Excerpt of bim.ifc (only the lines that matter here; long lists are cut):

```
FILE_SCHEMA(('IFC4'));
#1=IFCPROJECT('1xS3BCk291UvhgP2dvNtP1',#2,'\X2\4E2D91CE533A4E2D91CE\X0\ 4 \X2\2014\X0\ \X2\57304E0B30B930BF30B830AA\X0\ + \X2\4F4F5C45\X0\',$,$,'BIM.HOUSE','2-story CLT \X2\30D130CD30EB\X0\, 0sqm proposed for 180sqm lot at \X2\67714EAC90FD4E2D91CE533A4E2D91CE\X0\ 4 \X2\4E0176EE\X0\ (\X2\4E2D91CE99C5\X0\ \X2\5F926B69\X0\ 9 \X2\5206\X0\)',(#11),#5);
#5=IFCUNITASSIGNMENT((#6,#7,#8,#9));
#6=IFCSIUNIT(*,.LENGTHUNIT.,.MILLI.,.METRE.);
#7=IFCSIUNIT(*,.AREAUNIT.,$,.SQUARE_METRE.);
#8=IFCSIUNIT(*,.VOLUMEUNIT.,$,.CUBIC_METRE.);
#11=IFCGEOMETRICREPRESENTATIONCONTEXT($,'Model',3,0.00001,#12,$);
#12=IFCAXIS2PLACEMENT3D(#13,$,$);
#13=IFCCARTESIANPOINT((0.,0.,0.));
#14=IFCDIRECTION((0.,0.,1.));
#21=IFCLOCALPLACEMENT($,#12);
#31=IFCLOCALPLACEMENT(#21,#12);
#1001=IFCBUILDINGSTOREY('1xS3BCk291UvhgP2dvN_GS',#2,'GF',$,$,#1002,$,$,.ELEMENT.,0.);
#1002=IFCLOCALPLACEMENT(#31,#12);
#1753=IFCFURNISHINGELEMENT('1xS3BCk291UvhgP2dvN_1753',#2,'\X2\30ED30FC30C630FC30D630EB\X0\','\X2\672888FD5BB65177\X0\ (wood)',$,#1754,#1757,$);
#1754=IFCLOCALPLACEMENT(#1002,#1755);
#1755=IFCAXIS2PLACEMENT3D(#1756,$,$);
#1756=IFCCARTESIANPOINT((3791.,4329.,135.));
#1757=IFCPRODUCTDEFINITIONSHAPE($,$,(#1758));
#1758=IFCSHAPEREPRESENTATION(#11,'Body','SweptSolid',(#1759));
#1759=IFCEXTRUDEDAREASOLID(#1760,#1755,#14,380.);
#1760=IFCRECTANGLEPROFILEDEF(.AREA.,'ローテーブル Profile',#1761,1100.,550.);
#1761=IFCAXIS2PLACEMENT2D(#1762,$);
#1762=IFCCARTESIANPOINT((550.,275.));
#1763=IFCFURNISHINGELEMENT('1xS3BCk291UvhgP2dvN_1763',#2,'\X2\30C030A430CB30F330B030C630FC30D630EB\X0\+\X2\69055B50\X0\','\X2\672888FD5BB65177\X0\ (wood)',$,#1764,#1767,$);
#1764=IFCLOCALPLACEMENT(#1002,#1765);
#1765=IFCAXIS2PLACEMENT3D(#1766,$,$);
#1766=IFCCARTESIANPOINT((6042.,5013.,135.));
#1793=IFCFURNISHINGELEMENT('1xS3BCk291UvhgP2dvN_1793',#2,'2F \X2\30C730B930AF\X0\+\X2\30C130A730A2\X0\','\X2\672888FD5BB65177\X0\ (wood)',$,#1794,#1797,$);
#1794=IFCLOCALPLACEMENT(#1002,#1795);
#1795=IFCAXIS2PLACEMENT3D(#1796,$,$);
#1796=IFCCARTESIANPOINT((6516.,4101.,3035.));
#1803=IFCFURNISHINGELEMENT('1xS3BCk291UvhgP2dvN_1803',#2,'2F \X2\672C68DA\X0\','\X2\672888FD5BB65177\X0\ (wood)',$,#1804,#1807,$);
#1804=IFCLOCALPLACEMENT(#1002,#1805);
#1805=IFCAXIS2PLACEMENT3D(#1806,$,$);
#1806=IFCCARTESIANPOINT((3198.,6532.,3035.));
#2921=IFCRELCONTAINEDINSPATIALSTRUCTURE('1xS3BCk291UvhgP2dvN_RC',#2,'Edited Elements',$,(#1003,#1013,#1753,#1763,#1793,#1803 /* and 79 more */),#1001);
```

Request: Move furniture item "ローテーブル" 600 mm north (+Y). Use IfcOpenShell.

```python
import ifcopenshell
import ifcopenshell.api.geometry
import ifcopenshell.util.placement

model = ifcopenshell.open("bim.ifc")

item = model.by_guid("1xS3BCk291UvhgP2dvN_1753")
matrix = ifcopenshell.util.placement.get_local_placement(item.ObjectPlacement)
matrix[1, 3] += 600.0
ifcopenshell.api.geometry.edit_object_placement(model, product=item, matrix=matrix, is_si=False)

print(ifcopenshell.util.placement.get_local_placement(item.ObjectPlacement).round(3) + 0.0)

model.write("bim_rev.ifc")
```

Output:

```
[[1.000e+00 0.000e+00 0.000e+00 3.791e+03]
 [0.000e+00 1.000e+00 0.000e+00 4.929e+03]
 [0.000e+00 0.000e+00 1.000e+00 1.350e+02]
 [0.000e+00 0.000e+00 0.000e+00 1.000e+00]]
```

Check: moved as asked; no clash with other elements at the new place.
